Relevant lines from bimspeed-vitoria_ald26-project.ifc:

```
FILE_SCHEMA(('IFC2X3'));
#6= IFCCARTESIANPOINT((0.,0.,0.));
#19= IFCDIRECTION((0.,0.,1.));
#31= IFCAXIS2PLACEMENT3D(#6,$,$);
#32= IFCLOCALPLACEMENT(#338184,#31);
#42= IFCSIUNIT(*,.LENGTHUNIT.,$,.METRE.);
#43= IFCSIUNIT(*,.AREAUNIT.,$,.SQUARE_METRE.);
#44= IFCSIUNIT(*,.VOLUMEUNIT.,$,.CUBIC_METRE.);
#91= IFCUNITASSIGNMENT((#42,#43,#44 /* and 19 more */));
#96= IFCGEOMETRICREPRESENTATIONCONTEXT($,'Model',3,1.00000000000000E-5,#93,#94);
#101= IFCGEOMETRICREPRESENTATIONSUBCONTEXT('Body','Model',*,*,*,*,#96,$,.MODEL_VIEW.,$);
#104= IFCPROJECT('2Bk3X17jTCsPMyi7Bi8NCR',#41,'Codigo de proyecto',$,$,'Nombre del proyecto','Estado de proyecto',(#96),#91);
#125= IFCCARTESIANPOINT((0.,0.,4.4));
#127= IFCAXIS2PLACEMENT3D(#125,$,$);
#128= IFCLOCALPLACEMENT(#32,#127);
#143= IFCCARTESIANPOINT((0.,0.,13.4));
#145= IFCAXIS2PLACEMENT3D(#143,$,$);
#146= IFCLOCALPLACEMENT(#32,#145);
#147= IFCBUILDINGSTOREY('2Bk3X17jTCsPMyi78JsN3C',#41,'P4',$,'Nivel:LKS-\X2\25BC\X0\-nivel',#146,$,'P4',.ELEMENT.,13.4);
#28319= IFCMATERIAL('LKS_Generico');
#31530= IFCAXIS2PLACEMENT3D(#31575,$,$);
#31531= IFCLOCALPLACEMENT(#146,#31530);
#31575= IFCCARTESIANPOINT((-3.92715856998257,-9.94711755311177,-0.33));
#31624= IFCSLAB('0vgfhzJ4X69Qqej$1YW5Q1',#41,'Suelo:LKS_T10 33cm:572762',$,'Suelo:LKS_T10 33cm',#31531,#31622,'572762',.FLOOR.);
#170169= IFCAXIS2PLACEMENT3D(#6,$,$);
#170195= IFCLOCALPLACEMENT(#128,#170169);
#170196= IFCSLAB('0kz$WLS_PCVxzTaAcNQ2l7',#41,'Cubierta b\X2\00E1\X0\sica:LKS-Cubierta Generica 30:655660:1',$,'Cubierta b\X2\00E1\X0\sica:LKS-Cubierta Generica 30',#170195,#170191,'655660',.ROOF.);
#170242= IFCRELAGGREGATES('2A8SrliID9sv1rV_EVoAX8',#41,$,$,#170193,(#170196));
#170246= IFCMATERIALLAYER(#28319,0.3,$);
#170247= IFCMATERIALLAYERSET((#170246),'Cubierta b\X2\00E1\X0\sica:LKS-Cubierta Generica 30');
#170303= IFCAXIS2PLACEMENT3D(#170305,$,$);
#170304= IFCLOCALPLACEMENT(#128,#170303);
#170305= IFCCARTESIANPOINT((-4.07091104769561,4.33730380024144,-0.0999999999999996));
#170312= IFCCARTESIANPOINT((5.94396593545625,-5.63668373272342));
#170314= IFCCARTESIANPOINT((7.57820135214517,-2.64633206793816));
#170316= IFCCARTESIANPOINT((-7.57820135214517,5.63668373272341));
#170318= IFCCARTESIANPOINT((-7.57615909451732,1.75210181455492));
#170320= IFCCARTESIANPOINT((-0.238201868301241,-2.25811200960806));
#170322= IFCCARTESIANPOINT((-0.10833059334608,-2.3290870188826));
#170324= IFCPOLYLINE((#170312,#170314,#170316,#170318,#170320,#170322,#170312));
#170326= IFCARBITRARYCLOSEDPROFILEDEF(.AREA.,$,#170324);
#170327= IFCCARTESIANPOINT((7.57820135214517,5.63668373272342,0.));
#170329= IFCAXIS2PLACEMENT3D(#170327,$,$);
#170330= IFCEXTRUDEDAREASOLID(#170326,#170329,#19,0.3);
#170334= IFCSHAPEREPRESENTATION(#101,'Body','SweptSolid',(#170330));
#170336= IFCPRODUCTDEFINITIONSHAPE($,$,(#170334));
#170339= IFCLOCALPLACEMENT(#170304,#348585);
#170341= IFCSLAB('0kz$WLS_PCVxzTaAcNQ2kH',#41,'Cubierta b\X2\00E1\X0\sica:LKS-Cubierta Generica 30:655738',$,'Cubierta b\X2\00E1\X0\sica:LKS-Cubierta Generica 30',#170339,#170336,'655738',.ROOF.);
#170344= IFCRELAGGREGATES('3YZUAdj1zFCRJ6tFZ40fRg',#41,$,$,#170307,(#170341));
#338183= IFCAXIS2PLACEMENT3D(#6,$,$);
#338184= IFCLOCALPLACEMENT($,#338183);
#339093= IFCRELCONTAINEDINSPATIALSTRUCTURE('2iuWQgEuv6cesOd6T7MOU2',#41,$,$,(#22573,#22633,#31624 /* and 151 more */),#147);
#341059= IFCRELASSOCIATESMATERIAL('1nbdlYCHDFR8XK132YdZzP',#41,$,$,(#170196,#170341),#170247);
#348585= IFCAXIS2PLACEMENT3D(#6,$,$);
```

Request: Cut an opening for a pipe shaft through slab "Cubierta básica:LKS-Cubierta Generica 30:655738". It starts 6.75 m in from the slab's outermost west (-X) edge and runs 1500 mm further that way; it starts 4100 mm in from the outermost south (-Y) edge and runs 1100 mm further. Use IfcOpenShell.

```python
import numpy as np
import ifcopenshell
import ifcopenshell.api.feature
import ifcopenshell.api.geometry
import ifcopenshell.api.root
import ifcopenshell.geom
import ifcopenshell.util.placement
import ifcopenshell.util.representation
import ifcopenshell.util.shape
import ifcopenshell.util.unit

model = ifcopenshell.open("bimspeed-vitoria_ald26-project.ifc")
unit_scale = ifcopenshell.util.unit.calculate_unit_scale(model)
settings = ifcopenshell.geom.settings()


def volume(element):
    """Net volume in cubic metres, openings subtracted."""
    shape = ifcopenshell.geom.create_shape(settings, element)
    return ifcopenshell.util.shape.get_volume(shape.geometry)


slab = model.by_id(170341)
before = volume(slab)

# Extent in the slab's own axes, in metres. The edges named are its -X and -Y sides.
slab_shape = ifcopenshell.geom.create_shape(settings, slab)
vertices = ifcopenshell.util.shape.get_vertices(slab_shape.geometry)
x_min, y_min, bottom = vertices.min(axis=0)
top = vertices[:, 2].max()

opening = ifcopenshell.api.root.create_entity(model, ifc_class="IfcOpeningElement", name="Pipe shaft opening")
context = ifcopenshell.util.representation.get_context(model, "Model", "Body", "MODEL_VIEW")
width, depth = 1.5, 1.1
outline = [(0.0, 0.0), (width, 0.0), (width, depth), (0.0, depth), (0.0, 0.0)]
# Overshoot both faces by 50 mm so the cut is clean.
shape = ifcopenshell.api.geometry.add_slab_representation(
    model, context=context, depth=top - bottom + 0.1, polyline=outline
)
ifcopenshell.api.geometry.assign_representation(model, product=opening, representation=shape)

matrix = ifcopenshell.util.placement.get_local_placement(slab.ObjectPlacement)
matrix[:, 3] = matrix @ np.append(np.array([x_min + 6.75, y_min + 4.1, bottom - 0.05]) / unit_scale, 1.0)
ifcopenshell.api.geometry.edit_object_placement(model, product=opening, matrix=matrix, is_si=False)
ifcopenshell.api.feature.add_feature(model, feature=opening, element=slab)

after = volume(slab)

print(f"slab volume {before:.3f} -> {after:.3f} m3")

model.write("bimspeed-vitoria_ald26-project_edited.ifc")
```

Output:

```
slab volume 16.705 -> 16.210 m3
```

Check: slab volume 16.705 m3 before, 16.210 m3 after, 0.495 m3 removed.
